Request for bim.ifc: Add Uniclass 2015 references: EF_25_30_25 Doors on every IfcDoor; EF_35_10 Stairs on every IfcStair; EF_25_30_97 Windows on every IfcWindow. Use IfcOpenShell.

First a look at what the model holds.

```python
import ifcopenshell

model = ifcopenshell.open("bim.ifc")
print(model.schema)
print("classifications:", [c.Name for c in model.by_type("IfcClassification")])
for ifc_class in ("IfcDoor", "IfcRoof", "IfcStair", "IfcWall", "IfcWindow"):
    print(ifc_class, len(model.by_type(ifc_class)))
```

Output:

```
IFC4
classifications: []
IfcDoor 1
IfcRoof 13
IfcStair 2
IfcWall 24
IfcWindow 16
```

```python
import ifcopenshell
import ifcopenshell.api.classification

model = ifcopenshell.open("bim.ifc")

system = ifcopenshell.api.classification.add_classification(model, classification="Uniclass 2015")

codes = {
    "IfcDoor": ("EF_25_30_25", "Doors"),
    "IfcStair": ("EF_35_10", "Stairs"),
    "IfcWindow": ("EF_25_30_97", "Windows"),
}
for ifc_class, (code, name) in codes.items():
    products = model.by_type(ifc_class)
    ifcopenshell.api.classification.add_reference(
        model, products=products, classification=system, identification=code, name=name
    )
    print(code, len(products))

model.write("bim_updated.ifc")
```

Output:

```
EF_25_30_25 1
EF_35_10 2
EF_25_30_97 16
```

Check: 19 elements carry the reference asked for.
